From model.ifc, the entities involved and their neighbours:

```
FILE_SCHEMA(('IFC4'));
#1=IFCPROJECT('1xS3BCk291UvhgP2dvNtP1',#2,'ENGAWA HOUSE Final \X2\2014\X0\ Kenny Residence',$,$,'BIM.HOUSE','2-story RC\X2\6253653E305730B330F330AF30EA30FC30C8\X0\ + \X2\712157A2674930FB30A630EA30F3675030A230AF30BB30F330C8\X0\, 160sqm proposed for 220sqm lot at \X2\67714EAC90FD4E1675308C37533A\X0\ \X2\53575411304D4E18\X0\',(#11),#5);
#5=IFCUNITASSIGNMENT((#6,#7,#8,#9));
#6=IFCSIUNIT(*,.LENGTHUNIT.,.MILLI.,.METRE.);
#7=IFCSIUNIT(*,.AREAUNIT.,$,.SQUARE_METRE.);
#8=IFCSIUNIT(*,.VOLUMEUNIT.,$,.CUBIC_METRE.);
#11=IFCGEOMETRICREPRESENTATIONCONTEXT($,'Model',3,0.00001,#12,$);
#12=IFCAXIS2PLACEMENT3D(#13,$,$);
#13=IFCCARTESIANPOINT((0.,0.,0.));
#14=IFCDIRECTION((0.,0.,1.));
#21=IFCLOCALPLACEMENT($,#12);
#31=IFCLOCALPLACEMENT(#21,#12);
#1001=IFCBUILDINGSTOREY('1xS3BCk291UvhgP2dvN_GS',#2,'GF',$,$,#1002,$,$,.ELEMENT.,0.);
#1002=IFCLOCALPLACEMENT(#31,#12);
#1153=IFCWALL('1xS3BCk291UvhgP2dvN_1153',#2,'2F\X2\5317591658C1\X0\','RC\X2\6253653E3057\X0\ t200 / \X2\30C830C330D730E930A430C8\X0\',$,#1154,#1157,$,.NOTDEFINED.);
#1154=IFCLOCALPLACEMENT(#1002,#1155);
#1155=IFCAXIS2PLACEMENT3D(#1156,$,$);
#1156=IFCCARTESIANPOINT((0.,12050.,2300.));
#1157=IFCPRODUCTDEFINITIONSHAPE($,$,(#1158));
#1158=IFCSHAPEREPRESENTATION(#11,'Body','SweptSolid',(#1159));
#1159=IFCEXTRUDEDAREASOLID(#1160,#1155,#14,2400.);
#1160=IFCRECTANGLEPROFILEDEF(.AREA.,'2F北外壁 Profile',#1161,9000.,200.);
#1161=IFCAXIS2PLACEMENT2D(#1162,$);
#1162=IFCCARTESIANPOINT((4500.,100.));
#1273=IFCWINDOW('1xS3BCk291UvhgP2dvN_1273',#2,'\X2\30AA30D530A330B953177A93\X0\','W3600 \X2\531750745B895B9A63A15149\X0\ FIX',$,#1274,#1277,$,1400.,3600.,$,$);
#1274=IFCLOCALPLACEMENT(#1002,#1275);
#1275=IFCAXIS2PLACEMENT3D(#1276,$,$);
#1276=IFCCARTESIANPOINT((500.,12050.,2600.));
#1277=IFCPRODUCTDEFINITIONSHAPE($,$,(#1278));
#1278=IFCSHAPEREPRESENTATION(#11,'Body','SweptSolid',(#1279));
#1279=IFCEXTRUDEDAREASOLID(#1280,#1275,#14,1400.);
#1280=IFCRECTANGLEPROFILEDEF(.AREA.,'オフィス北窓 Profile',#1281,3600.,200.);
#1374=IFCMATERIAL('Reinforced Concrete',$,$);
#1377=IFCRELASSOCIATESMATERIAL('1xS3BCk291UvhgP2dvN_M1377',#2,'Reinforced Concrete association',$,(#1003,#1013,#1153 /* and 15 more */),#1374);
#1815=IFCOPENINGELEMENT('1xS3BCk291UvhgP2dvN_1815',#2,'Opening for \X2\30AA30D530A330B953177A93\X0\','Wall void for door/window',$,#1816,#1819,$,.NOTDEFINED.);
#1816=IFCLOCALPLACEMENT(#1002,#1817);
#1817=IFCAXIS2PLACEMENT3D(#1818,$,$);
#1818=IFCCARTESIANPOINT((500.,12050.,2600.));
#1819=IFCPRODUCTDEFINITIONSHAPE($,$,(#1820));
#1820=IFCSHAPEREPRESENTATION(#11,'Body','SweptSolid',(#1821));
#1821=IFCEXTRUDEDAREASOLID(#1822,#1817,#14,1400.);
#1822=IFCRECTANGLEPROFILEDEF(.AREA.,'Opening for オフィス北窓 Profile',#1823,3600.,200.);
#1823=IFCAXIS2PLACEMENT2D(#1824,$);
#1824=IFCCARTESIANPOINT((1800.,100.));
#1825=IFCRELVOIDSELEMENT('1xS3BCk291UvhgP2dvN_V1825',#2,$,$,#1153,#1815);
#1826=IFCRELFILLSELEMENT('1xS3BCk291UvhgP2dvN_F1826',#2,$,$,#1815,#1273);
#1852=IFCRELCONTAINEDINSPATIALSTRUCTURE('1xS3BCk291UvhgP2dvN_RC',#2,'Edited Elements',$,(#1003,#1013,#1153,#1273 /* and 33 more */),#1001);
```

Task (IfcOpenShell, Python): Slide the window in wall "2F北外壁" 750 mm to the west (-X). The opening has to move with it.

```python
import ifcopenshell
import ifcopenshell.api.geometry
import ifcopenshell.util.placement
import ifcopenshell.util.unit

model = ifcopenshell.open("model.ifc")
unit_scale = ifcopenshell.util.unit.calculate_unit_scale(model)

window = model.by_id(1273)
opening = window.FillsVoids[0].RelatingOpeningElement
wall = opening.VoidsElements[0].RelatingBuildingElement

wall_matrix = ifcopenshell.util.placement.get_local_placement(wall.ObjectPlacement)
shift = wall_matrix[:3, 0] * -0.75 / unit_scale
before = ifcopenshell.util.placement.get_local_placement(window.ObjectPlacement)[:3, 3].copy()

# The window is not placed relative to its opening, so move both.
for product in (opening, window):
    matrix = ifcopenshell.util.placement.get_local_placement(product.ObjectPlacement)
    matrix[:3, 3] += shift
    ifcopenshell.api.geometry.edit_object_placement(model, product=product, matrix=matrix, is_si=False)

after = ifcopenshell.util.placement.get_local_placement(window.ObjectPlacement)[:3, 3]
print("window moved by", (after - before).round(3) + 0.0)

model.write("model_updated.ifc")
```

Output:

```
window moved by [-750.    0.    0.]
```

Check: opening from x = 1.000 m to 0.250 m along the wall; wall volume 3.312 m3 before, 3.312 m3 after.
